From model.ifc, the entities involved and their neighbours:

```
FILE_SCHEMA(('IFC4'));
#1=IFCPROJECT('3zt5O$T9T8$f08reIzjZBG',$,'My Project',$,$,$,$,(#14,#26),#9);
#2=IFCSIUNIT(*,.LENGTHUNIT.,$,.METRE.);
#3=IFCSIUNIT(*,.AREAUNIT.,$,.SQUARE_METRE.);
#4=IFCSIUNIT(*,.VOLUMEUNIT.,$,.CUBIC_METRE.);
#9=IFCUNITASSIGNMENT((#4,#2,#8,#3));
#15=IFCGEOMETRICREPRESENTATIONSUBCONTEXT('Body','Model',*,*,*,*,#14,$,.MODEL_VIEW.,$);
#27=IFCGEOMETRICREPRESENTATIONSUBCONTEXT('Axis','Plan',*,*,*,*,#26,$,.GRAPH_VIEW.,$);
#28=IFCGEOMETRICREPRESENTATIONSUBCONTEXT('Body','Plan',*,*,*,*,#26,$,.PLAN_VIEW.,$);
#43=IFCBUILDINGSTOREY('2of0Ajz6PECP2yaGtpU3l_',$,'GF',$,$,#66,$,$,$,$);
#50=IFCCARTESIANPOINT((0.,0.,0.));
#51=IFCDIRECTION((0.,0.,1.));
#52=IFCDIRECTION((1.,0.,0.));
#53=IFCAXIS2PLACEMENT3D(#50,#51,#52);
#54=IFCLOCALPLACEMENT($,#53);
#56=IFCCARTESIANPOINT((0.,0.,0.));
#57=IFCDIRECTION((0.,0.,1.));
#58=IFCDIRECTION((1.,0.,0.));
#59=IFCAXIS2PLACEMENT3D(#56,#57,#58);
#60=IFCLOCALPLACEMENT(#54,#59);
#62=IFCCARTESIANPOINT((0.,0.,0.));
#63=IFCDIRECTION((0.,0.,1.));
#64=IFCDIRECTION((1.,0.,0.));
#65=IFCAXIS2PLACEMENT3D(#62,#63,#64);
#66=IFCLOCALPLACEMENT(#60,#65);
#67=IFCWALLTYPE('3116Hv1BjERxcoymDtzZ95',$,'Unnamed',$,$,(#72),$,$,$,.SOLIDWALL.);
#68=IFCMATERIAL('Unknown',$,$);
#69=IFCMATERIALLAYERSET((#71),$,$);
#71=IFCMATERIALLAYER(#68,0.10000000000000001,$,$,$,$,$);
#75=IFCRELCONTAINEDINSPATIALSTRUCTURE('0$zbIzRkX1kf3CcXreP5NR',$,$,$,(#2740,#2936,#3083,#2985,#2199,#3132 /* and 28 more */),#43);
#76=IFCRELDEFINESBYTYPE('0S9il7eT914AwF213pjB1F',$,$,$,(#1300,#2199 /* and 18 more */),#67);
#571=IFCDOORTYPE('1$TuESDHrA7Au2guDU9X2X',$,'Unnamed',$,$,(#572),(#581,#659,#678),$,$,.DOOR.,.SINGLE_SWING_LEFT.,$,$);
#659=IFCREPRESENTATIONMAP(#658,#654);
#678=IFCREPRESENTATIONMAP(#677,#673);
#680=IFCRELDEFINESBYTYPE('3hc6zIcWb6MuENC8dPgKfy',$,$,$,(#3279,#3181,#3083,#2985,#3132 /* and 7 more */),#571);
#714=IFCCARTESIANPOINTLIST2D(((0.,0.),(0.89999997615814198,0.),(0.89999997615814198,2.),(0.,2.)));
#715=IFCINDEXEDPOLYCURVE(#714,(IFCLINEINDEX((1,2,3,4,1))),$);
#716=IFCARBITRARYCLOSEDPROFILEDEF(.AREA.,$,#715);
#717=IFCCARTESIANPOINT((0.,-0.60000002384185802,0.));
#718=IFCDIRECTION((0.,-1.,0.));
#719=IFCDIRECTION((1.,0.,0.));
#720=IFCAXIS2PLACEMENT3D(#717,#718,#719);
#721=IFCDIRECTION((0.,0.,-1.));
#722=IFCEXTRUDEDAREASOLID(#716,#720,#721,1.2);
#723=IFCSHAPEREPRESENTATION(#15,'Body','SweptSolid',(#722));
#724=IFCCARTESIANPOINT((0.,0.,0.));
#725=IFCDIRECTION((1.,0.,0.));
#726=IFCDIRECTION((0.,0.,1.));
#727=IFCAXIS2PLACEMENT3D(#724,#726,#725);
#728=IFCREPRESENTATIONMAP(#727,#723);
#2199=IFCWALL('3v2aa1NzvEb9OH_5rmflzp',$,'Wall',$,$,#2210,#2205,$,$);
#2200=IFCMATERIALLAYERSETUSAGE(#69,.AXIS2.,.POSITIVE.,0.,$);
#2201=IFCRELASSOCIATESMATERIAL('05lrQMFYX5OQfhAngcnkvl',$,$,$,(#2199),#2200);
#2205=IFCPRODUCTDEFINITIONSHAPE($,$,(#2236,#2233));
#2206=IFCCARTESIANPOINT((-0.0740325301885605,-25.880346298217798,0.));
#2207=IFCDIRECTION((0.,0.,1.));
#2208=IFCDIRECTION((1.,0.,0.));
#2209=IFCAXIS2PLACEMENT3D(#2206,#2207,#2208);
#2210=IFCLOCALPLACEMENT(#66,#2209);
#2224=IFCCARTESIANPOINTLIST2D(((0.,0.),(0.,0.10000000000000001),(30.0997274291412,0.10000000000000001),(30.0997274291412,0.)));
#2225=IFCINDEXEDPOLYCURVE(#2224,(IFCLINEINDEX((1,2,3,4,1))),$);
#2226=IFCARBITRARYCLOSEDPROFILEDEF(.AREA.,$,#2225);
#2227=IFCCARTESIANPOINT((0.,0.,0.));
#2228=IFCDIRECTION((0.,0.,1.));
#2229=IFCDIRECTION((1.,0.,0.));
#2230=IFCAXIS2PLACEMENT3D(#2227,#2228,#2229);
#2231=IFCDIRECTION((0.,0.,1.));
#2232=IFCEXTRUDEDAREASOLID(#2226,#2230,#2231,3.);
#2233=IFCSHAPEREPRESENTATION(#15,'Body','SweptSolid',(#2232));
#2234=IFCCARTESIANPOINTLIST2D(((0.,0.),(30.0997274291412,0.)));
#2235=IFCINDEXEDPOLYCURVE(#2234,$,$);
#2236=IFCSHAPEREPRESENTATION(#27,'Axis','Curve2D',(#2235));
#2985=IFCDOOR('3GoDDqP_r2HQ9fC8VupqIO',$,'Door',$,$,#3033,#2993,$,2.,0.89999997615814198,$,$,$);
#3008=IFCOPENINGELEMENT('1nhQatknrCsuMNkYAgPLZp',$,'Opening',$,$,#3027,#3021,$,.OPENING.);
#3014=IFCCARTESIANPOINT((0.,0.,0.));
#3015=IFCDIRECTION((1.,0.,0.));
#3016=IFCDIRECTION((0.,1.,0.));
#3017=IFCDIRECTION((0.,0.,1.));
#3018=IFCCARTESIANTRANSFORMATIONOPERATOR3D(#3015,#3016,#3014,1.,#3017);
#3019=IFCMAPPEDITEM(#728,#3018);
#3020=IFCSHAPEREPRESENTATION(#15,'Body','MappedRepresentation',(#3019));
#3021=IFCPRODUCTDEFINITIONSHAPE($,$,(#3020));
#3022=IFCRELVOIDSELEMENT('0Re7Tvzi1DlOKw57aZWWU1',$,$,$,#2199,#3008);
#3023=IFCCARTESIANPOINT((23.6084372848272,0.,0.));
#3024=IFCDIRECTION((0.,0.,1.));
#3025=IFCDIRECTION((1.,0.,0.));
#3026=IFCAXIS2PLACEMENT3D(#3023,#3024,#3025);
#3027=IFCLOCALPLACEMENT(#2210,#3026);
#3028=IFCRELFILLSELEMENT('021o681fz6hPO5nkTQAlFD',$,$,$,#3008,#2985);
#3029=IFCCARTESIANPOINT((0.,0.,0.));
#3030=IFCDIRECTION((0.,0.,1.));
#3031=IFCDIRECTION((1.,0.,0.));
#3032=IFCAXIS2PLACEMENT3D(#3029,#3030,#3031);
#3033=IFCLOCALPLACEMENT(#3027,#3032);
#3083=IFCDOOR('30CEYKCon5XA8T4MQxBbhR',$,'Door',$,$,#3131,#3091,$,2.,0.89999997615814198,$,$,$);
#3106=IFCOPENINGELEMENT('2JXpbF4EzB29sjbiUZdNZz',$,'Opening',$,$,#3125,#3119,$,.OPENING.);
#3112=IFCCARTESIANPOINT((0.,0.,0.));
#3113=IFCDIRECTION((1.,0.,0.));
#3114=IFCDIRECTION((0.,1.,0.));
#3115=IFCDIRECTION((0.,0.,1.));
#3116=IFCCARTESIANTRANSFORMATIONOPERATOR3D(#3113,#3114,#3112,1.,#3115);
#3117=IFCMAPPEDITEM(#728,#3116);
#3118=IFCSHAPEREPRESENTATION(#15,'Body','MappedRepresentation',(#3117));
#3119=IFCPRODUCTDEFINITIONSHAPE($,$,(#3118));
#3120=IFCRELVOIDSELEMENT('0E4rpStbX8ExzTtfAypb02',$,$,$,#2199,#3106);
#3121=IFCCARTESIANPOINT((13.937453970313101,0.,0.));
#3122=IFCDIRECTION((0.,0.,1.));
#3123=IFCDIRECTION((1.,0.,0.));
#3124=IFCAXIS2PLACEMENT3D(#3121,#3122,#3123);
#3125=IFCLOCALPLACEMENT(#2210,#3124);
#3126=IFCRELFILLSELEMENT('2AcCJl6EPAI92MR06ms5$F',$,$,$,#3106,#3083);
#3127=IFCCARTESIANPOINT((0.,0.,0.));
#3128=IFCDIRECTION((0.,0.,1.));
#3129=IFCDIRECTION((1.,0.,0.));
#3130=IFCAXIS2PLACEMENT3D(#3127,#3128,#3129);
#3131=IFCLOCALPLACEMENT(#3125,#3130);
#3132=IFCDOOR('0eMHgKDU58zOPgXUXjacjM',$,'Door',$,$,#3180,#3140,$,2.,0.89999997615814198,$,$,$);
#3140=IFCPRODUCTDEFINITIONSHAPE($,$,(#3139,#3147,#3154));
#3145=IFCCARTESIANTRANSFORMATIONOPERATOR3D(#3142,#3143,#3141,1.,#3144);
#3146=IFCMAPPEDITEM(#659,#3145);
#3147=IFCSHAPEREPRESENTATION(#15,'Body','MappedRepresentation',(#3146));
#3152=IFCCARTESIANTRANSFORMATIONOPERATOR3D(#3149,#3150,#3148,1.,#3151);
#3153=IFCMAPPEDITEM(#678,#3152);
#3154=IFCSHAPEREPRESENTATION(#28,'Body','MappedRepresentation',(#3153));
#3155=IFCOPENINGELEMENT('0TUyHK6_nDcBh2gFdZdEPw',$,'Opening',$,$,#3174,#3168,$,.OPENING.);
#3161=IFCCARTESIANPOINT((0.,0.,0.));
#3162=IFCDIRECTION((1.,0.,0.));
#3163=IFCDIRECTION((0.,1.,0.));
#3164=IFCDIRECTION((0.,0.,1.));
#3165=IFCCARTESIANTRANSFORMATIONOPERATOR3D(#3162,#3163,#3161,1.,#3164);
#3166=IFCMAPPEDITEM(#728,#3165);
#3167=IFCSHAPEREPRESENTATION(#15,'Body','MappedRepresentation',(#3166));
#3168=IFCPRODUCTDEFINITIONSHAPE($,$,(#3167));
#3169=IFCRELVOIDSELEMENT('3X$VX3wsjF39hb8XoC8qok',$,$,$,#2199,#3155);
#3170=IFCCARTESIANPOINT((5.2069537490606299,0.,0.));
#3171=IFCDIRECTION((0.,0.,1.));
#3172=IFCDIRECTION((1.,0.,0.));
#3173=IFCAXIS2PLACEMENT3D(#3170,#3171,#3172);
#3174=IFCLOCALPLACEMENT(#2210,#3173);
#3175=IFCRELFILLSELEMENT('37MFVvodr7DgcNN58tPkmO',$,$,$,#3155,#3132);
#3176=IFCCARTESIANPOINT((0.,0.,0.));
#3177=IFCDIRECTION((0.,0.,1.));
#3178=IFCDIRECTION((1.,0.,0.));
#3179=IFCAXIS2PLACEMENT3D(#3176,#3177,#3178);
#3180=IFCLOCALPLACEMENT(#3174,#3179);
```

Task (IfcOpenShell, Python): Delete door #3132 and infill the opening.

```python
import ifcopenshell
import ifcopenshell.api.feature
import ifcopenshell.api.root
import ifcopenshell.geom
import ifcopenshell.util.shape

model = ifcopenshell.open("model.ifc")
settings = ifcopenshell.geom.settings()


def volume(element):
    """Net volume in cubic metres, openings subtracted."""
    shape = ifcopenshell.geom.create_shape(settings, element)
    return ifcopenshell.util.shape.get_volume(shape.geometry)


door = model.by_guid("0eMHgKDU58zOPgXUXjacjM")
opening = door.FillsVoids[0].RelatingOpeningElement
wall = opening.VoidsElements[0].RelatingBuildingElement
before = volume(wall)

ifcopenshell.api.root.remove_product(model, product=door)
ifcopenshell.api.feature.remove_feature(model, feature=opening)

after = volume(wall)

print(f"wall volume {before:.3f} -> {after:.3f} m3")

model.write("model_rev.ifc")
```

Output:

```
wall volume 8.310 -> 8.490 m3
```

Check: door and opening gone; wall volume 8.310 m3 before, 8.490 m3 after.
